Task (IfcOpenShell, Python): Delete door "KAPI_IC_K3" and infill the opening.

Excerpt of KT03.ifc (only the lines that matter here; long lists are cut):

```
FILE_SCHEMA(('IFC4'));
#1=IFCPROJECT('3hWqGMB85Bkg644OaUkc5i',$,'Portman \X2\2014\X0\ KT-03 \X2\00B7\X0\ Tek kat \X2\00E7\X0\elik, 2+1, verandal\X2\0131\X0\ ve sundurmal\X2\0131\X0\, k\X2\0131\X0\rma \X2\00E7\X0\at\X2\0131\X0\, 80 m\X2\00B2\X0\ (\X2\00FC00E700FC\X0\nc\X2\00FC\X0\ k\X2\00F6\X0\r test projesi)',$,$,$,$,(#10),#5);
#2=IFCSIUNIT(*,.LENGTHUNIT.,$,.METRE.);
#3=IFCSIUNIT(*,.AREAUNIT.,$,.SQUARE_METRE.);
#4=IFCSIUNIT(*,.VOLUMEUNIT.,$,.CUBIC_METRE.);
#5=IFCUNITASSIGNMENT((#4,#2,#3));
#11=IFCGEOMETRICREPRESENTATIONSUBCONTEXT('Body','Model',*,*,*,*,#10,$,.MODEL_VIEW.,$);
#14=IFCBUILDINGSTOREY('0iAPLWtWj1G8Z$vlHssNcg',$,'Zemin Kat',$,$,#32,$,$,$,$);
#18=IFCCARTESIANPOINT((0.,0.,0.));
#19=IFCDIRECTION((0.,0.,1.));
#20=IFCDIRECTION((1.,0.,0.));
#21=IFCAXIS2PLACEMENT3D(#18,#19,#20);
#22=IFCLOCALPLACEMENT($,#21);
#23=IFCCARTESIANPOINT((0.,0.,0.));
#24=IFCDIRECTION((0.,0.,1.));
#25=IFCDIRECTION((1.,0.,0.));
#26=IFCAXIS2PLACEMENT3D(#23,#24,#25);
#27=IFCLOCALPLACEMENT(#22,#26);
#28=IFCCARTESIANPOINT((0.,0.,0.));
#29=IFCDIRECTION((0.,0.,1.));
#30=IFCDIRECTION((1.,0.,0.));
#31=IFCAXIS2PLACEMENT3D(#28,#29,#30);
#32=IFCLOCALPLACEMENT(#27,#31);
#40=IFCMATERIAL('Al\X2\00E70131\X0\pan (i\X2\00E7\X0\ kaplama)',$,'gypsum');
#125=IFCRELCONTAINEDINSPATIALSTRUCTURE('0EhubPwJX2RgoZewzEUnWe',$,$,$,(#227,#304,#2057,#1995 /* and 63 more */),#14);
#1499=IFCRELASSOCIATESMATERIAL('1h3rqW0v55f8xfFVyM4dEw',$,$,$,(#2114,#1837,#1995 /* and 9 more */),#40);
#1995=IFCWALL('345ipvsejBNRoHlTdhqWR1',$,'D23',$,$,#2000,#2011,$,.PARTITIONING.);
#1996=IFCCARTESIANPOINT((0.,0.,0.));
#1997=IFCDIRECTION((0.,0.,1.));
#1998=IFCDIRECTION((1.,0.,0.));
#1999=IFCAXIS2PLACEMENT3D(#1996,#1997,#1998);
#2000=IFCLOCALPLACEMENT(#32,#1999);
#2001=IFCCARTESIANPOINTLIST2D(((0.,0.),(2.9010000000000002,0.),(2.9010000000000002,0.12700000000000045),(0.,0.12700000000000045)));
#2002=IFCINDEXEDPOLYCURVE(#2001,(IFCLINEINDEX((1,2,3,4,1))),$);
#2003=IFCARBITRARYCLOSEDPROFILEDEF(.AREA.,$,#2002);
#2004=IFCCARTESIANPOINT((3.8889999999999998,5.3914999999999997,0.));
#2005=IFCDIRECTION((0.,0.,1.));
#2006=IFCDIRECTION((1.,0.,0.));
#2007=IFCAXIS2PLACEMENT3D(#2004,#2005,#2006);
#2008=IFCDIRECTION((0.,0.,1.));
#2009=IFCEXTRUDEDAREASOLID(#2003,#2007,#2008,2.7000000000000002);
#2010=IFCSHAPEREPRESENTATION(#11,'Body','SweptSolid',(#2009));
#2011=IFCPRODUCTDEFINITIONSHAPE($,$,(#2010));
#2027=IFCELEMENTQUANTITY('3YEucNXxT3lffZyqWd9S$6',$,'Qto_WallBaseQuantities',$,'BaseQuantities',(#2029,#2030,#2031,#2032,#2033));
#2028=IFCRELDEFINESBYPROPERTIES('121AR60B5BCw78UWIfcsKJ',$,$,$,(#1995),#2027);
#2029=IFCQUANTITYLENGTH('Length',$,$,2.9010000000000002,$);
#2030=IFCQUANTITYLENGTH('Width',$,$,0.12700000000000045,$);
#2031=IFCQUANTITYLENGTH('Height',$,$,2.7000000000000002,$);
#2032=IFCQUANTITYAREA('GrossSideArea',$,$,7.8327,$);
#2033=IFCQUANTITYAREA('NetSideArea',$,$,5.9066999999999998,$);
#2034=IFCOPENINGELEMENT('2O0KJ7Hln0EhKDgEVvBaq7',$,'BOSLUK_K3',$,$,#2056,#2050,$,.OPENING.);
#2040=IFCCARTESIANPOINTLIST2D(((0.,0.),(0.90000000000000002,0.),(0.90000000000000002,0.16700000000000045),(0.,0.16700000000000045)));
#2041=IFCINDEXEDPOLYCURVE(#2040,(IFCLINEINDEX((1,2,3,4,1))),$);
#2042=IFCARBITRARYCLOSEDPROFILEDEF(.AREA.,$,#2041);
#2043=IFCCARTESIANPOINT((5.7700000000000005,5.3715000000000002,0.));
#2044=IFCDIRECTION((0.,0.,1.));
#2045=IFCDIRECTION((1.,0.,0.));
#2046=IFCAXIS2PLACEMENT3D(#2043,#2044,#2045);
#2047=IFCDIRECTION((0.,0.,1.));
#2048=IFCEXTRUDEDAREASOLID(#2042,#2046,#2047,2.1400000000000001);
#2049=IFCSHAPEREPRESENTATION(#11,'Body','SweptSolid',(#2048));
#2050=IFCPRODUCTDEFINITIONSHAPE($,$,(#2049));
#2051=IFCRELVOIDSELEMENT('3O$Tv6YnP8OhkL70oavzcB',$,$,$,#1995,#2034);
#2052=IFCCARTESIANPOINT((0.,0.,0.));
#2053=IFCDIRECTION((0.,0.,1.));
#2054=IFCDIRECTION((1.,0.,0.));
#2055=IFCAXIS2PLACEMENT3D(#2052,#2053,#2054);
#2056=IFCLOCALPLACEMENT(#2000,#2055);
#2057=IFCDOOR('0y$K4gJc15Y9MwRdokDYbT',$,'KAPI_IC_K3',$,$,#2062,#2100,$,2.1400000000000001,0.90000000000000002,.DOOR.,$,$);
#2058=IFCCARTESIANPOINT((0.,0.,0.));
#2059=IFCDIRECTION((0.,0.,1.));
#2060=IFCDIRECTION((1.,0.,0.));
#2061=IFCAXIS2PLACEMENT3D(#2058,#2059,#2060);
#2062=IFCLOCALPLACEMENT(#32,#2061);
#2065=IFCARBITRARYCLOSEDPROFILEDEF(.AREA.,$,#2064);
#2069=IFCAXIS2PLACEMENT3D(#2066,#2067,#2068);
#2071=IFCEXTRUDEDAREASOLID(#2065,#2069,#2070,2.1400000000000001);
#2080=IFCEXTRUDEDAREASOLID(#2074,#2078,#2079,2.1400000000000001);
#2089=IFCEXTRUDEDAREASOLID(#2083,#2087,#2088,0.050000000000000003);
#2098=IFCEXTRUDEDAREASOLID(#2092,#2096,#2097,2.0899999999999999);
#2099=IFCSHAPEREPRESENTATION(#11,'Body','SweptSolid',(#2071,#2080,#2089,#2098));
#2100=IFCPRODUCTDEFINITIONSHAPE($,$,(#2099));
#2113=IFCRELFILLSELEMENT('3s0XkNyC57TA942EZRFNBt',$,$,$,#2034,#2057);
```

```python
import ifcopenshell
import ifcopenshell.api.feature
import ifcopenshell.api.pset
import ifcopenshell.api.root
import ifcopenshell.geom
import ifcopenshell.util.element
import ifcopenshell.util.shape
import ifcopenshell.util.unit

model = ifcopenshell.open("KT03.ifc")
area_scale = ifcopenshell.util.unit.calculate_unit_scale(model, "AREAUNIT")
settings = ifcopenshell.geom.settings()


def volume(element):
    """Net volume in cubic metres, openings subtracted."""
    shape = ifcopenshell.geom.create_shape(settings, element)
    return ifcopenshell.util.shape.get_volume(shape.geometry)


door = model.by_id(2057)
opening = door.FillsVoids[0].RelatingOpeningElement
wall = opening.VoidsElements[0].RelatingBuildingElement
before = volume(wall)

ifcopenshell.api.root.remove_product(model, product=door)
ifcopenshell.api.feature.remove_feature(model, feature=opening)

after = volume(wall)
thickness = 0.127  # wall thickness in metres

# Update the wall's stored quantities.
qto = model.by_id(ifcopenshell.util.element.get_pset(wall, "Qto_WallBaseQuantities", should_inherit=False)["id"])
ifcopenshell.api.pset.edit_qto(model, qto=qto, properties={"NetSideArea": after / thickness / area_scale})

print(f"wall volume {before:.3f} -> {after:.3f} m3")

model.write("KT03_rev.ifc")
```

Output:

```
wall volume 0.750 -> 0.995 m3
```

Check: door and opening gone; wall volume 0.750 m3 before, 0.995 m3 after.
